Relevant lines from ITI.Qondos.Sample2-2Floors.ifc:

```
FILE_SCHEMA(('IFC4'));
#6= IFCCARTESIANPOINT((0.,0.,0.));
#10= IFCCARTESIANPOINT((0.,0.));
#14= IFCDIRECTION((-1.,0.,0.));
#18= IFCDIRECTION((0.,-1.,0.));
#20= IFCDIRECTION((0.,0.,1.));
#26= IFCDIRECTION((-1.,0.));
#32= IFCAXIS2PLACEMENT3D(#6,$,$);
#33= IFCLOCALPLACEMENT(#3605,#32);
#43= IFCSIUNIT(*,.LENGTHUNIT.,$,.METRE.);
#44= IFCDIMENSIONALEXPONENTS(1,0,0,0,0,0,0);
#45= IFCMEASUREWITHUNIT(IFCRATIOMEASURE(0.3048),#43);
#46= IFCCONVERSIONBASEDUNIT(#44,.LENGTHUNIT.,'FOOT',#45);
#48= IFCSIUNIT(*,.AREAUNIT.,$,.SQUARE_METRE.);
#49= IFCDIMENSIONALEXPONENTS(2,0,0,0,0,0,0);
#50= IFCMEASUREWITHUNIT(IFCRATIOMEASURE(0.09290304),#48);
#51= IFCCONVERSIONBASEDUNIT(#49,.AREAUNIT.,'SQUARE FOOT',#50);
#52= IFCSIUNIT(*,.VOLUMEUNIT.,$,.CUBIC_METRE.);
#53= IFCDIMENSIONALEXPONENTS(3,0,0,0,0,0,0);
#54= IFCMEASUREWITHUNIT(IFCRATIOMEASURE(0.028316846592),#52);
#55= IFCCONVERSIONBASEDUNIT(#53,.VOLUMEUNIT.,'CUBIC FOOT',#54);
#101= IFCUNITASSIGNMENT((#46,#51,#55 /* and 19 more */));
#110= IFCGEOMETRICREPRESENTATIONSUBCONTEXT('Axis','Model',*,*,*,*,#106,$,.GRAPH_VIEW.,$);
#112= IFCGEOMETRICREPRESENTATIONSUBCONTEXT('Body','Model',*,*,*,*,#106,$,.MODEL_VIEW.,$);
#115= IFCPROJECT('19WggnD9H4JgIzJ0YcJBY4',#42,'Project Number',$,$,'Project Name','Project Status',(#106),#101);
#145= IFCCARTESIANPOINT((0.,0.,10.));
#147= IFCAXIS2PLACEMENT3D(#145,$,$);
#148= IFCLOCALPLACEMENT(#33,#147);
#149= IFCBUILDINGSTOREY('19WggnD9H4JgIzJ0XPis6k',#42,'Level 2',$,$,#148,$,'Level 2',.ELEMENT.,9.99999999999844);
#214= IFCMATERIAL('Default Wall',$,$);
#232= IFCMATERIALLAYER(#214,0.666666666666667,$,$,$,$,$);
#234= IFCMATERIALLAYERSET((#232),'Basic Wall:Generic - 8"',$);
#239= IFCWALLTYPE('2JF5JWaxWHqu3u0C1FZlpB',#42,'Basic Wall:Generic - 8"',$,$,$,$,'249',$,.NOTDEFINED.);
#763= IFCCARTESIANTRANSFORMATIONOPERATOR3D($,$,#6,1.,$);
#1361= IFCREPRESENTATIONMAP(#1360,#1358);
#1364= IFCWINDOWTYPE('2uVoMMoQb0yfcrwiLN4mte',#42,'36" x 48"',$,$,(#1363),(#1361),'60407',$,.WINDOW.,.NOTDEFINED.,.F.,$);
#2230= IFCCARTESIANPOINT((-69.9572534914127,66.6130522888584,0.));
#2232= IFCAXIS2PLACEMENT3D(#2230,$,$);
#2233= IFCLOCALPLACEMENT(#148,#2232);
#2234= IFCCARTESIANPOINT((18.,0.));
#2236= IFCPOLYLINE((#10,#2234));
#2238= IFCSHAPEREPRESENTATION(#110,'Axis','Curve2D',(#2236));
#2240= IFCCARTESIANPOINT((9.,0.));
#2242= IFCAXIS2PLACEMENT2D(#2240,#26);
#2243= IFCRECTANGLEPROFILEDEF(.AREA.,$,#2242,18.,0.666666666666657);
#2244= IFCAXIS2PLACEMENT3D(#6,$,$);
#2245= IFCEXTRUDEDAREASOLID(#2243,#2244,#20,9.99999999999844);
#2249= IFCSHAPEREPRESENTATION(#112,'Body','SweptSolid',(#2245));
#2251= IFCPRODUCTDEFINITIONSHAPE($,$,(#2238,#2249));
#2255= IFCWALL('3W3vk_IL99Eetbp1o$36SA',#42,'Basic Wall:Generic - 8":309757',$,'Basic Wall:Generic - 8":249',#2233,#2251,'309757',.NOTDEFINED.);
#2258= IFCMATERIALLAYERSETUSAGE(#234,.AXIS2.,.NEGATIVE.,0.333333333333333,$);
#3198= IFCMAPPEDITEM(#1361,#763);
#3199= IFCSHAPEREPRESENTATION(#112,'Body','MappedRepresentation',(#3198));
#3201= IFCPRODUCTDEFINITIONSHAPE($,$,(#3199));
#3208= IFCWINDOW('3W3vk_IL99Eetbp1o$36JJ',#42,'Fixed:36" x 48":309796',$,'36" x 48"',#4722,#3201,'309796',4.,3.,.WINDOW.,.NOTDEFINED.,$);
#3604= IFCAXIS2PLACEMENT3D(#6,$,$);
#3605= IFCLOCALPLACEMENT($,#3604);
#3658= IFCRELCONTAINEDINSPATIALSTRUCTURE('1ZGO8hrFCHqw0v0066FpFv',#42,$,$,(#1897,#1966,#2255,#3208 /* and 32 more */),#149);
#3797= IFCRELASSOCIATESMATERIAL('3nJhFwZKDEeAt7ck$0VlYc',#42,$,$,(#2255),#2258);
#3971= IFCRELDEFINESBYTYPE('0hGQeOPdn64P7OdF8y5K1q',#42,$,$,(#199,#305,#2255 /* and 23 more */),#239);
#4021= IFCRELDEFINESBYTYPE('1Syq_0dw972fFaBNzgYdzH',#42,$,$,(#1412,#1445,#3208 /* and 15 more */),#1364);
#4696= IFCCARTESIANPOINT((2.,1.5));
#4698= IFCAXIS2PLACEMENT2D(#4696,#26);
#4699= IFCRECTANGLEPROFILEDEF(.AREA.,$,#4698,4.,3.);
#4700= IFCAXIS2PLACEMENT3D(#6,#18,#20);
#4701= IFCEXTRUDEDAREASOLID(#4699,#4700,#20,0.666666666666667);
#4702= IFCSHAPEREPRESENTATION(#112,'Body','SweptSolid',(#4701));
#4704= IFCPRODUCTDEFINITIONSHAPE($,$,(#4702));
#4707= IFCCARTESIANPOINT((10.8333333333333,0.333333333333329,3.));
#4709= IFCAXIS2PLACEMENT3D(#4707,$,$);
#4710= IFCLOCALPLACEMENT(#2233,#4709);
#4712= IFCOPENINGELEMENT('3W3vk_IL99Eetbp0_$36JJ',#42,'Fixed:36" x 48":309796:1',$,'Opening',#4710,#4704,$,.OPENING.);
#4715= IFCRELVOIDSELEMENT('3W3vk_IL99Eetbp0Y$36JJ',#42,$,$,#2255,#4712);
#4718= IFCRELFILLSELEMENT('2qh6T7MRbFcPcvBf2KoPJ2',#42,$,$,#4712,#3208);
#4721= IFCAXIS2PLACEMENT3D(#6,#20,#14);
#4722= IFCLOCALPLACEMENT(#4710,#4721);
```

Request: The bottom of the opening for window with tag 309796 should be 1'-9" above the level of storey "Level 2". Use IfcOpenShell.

```python
import numpy as np
import ifcopenshell
import ifcopenshell.api.geometry
import ifcopenshell.geom
import ifcopenshell.util.element
import ifcopenshell.util.placement
import ifcopenshell.util.shape
import ifcopenshell.util.unit

model = ifcopenshell.open("ITI.Qondos.Sample2-2Floors.ifc")
unit_scale = ifcopenshell.util.unit.calculate_unit_scale(model)

window = model.by_guid("3W3vk_IL99Eetbp1o$36JJ")
opening = window.FillsVoids[0].RelatingOpeningElement
storey = ifcopenshell.util.element.get_container(window, ifc_class="IfcBuildingStorey")
level = ifcopenshell.util.placement.get_local_placement(storey.ObjectPlacement)[2, 3]

# The opening's origin need not be at the sill, so measure its lowest point.
shape = ifcopenshell.geom.create_shape(ifcopenshell.geom.settings(), opening)
bottom = ifcopenshell.util.shape.get_shape_bottom_elevation(shape, shape.geometry) / unit_scale
dz = level + 21 * 0.0254 / unit_scale - bottom

shift = np.array([0.0, 0.0, dz])
# The window is placed relative to its opening, so it follows when the opening moves.
matrix = ifcopenshell.util.placement.get_local_placement(opening.ObjectPlacement)
matrix[:3, 3] += shift
ifcopenshell.api.geometry.edit_object_placement(
    model, product=opening, matrix=matrix, is_si=False, should_transform_children=True
)

print(f"moved by {dz * unit_scale:+.3f} m")

model.write("ITI.Qondos.Sample2-2Floors_rev.ifc")
```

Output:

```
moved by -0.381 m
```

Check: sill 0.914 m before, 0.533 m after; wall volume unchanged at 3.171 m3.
